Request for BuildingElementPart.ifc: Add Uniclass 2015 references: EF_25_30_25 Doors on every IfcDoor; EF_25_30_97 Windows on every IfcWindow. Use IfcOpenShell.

First a look at what the model holds.

```python
import ifcopenshell

model = ifcopenshell.open("BuildingElementPart.ifc")
print(model.schema)
print("classifications:", [c.Name for c in model.by_type("IfcClassification")])
for ifc_class in ("IfcDoor", "IfcRoof", "IfcStair", "IfcWall", "IfcWindow"):
    print(ifc_class, len(model.by_type(ifc_class)))
```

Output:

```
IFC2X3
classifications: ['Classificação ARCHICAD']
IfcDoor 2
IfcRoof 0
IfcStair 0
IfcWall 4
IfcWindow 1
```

```python
import ifcopenshell
import ifcopenshell.api.classification

model = ifcopenshell.open("BuildingElementPart.ifc")

# IFC2X3 requires Source and Edition and has no link from the project to the system.
system = model.create_entity("IfcClassification", Source="NBS", Edition="2015", Name="Uniclass 2015")

codes = {
    "IfcDoor": ("EF_25_30_25", "Doors"),
    "IfcWindow": ("EF_25_30_97", "Windows"),
}
for ifc_class, (code, name) in codes.items():
    products = model.by_type(ifc_class)
    ifcopenshell.api.classification.add_reference(
        model, products=products, classification=system, identification=code, name=name
    )
    print(code, len(products))

model.write("BuildingElementPart_v2.ifc")
```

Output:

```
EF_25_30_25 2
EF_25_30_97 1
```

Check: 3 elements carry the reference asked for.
